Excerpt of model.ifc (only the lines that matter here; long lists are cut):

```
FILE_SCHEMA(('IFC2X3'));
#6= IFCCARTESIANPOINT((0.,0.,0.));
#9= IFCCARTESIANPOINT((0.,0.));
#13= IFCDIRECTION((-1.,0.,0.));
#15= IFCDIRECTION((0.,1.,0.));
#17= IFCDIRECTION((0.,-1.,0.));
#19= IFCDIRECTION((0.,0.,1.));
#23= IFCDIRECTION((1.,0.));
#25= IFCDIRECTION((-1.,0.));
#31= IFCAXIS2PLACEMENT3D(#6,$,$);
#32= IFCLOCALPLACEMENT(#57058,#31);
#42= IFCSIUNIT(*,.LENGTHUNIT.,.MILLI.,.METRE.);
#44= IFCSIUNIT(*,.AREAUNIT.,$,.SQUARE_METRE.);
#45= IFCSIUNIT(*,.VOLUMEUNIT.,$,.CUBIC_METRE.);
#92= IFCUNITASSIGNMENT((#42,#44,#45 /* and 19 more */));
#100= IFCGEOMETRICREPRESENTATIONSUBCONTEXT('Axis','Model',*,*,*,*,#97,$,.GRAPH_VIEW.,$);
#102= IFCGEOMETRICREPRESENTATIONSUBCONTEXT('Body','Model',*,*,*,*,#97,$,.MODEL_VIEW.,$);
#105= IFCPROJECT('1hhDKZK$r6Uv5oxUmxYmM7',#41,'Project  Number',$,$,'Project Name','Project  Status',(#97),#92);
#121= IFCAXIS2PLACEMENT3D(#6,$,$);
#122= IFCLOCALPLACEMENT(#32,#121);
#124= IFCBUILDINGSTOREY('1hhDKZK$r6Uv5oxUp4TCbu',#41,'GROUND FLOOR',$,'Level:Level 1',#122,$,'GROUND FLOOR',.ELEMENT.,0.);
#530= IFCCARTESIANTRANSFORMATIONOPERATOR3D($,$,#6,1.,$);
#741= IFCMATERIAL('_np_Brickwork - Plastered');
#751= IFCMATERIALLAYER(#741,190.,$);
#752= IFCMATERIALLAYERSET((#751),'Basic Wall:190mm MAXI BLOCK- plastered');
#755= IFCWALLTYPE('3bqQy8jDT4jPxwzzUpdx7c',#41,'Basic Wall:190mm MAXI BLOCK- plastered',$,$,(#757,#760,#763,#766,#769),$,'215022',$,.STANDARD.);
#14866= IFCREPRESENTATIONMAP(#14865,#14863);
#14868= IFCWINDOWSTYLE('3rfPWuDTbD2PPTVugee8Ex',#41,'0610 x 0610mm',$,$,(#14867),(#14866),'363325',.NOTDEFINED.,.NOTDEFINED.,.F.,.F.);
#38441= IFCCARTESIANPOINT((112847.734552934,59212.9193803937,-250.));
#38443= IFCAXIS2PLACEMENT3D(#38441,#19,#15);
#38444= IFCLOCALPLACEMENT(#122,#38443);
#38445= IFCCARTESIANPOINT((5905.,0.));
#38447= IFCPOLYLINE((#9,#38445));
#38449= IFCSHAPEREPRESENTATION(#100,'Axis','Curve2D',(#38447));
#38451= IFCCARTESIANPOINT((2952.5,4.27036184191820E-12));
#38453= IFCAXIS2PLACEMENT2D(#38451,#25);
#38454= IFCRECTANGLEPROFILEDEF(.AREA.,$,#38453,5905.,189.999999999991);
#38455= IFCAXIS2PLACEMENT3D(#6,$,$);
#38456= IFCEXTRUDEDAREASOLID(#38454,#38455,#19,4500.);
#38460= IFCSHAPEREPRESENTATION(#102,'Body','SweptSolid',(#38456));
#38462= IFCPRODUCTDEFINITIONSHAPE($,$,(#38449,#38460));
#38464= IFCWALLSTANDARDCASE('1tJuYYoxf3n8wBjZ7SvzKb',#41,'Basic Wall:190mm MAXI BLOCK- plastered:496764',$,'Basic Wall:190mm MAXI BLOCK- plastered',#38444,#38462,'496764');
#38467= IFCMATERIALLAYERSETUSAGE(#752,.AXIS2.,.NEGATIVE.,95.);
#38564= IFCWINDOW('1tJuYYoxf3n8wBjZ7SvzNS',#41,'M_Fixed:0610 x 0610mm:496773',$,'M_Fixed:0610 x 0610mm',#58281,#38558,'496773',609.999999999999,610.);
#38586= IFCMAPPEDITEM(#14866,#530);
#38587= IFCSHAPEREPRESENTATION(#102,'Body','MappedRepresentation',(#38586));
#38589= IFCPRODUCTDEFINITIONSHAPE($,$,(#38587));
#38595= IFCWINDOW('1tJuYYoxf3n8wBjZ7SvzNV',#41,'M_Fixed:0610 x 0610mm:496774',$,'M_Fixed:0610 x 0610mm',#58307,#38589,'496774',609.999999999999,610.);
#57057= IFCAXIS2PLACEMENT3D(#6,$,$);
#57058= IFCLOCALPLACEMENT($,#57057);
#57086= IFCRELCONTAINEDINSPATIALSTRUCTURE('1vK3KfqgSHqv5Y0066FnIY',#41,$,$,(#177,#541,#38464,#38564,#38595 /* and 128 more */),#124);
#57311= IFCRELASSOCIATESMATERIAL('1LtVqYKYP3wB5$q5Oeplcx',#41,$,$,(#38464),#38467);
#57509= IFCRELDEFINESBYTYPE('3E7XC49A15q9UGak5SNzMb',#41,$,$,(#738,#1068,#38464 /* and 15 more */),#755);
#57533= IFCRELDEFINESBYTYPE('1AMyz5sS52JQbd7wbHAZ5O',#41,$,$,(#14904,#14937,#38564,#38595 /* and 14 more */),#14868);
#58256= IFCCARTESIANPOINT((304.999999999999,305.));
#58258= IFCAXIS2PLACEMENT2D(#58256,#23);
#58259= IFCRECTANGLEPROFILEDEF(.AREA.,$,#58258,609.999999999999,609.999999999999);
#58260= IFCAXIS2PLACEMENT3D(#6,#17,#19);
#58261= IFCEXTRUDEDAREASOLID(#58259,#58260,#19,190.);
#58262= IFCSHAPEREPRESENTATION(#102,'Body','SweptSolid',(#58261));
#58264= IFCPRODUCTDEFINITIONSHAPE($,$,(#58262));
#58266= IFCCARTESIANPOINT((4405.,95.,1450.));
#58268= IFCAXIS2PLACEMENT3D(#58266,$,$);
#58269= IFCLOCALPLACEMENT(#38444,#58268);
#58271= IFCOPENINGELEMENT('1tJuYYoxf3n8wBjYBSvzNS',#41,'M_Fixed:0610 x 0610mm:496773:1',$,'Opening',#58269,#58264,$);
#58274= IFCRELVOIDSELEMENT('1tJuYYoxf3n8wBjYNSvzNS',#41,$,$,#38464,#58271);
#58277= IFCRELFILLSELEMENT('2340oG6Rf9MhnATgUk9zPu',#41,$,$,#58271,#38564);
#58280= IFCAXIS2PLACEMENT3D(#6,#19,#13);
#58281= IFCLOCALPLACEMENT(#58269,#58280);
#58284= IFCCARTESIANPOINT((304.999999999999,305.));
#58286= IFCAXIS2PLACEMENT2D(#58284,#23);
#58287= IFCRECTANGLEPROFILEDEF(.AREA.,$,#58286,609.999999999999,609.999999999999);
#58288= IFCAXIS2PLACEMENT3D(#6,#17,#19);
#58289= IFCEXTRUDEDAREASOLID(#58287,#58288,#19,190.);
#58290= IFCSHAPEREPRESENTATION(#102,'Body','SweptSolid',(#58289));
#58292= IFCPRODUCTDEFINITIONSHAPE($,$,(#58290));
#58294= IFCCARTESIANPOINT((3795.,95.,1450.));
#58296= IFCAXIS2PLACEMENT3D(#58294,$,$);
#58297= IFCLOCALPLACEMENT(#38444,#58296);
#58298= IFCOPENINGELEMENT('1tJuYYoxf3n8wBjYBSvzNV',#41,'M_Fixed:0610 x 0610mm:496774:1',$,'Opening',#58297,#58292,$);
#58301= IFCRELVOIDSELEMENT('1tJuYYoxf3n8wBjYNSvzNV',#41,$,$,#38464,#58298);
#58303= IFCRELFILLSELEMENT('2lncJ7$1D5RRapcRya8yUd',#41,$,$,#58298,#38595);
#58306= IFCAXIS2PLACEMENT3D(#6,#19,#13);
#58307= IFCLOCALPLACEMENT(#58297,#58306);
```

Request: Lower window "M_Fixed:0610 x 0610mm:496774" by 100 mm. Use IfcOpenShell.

```python
import numpy as np
import ifcopenshell
import ifcopenshell.api.geometry
import ifcopenshell.util.placement
import ifcopenshell.util.unit

model = ifcopenshell.open("model.ifc")
unit_scale = ifcopenshell.util.unit.calculate_unit_scale(model)

window = model.by_guid("1tJuYYoxf3n8wBjZ7SvzNV")
opening = window.FillsVoids[0].RelatingOpeningElement
dz = -0.1 / unit_scale

shift = np.array([0.0, 0.0, dz])
# The window is placed relative to its opening, so it follows when the opening moves.
matrix = ifcopenshell.util.placement.get_local_placement(opening.ObjectPlacement)
matrix[:3, 3] += shift
ifcopenshell.api.geometry.edit_object_placement(
    model, product=opening, matrix=matrix, is_si=False, should_transform_children=True
)

print(f"moved by {dz * unit_scale:+.3f} m")

model.write("model_v2.ifc")
```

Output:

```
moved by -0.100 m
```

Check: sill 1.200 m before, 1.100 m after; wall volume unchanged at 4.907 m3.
